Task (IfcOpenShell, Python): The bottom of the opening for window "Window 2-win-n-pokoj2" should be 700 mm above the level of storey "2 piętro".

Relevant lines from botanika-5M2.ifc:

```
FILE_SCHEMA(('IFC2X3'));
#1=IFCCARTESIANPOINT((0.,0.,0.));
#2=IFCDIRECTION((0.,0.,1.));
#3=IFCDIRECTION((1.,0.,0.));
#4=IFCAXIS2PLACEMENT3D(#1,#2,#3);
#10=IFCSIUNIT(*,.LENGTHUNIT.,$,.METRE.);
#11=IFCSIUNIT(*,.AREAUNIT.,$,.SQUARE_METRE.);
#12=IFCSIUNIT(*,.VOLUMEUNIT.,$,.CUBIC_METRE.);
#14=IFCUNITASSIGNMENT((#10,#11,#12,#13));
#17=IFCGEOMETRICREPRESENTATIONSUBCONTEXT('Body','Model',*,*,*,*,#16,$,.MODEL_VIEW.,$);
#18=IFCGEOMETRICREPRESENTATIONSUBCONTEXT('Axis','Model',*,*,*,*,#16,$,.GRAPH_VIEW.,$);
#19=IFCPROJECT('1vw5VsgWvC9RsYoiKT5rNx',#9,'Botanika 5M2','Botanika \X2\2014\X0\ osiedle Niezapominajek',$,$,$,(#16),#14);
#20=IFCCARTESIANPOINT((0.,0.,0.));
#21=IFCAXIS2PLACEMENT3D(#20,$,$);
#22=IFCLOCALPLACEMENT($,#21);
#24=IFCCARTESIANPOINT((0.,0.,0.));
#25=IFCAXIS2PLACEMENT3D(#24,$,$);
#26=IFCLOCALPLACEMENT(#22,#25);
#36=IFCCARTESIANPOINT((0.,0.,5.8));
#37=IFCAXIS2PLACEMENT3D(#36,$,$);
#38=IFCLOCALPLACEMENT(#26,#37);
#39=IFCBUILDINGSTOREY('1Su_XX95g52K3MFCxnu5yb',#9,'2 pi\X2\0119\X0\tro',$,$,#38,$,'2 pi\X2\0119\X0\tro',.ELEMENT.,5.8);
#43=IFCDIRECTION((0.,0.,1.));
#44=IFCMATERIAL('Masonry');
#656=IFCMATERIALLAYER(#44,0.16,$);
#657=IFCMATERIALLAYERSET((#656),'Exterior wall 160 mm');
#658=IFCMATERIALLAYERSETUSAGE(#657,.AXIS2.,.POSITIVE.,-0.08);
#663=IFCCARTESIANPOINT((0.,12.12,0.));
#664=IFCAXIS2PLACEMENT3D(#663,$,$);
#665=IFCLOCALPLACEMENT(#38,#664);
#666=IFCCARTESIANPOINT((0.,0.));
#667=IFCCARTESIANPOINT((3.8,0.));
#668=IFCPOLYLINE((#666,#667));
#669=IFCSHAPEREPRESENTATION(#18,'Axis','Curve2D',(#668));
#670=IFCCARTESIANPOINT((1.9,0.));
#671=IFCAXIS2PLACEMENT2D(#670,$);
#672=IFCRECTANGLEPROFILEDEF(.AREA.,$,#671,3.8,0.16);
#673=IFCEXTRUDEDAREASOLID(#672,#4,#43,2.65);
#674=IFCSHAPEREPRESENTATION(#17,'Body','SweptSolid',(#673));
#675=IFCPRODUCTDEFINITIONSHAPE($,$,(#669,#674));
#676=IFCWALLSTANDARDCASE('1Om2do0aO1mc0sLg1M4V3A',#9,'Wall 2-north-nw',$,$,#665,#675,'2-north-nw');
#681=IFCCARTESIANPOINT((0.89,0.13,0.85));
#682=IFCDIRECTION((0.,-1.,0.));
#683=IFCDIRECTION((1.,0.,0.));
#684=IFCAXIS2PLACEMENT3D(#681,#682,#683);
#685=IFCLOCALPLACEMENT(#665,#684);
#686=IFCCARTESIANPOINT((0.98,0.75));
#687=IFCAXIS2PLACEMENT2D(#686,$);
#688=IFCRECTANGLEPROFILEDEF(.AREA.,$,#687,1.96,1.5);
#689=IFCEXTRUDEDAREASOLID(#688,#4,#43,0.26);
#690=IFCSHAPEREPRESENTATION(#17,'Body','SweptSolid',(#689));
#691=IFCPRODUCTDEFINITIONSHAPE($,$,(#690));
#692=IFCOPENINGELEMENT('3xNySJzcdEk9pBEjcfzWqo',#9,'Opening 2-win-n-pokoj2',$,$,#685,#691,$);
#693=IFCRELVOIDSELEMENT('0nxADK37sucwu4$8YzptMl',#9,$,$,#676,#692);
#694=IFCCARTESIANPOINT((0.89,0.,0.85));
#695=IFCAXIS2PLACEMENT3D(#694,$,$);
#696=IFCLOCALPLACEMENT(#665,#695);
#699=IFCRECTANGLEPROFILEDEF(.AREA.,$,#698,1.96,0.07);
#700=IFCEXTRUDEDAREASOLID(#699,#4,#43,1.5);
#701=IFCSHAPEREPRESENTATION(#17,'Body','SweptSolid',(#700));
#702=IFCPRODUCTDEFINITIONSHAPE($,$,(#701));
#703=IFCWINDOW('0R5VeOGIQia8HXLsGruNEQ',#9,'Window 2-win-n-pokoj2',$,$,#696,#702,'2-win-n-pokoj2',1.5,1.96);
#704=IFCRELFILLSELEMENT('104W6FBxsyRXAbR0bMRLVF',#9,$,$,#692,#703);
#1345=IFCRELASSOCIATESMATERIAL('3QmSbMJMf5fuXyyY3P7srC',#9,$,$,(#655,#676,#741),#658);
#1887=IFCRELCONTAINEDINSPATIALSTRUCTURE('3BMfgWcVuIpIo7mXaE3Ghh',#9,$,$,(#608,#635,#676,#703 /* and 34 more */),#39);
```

```python
import numpy as np
import ifcopenshell
import ifcopenshell.api.geometry
import ifcopenshell.geom
import ifcopenshell.util.element
import ifcopenshell.util.placement
import ifcopenshell.util.shape
import ifcopenshell.util.unit

model = ifcopenshell.open("botanika-5M2.ifc")
unit_scale = ifcopenshell.util.unit.calculate_unit_scale(model)

window = model.by_guid("0R5VeOGIQia8HXLsGruNEQ")
opening = window.FillsVoids[0].RelatingOpeningElement
storey = ifcopenshell.util.element.get_container(window, ifc_class="IfcBuildingStorey")
level = ifcopenshell.util.placement.get_local_placement(storey.ObjectPlacement)[2, 3]

# The opening's origin need not be at the sill, so measure its lowest point.
shape = ifcopenshell.geom.create_shape(ifcopenshell.geom.settings(), opening)
bottom = ifcopenshell.util.shape.get_shape_bottom_elevation(shape, shape.geometry) / unit_scale
dz = level + 0.7 / unit_scale - bottom

shift = np.array([0.0, 0.0, dz])
# The window is not placed relative to its opening, so move both.
for product in (opening, window):
    matrix = ifcopenshell.util.placement.get_local_placement(product.ObjectPlacement)
    matrix[:3, 3] += shift
    ifcopenshell.api.geometry.edit_object_placement(model, product=product, matrix=matrix, is_si=False)

print(f"moved by {dz * unit_scale:+.3f} m")

model.write("botanika-5M2_rev.ifc")
```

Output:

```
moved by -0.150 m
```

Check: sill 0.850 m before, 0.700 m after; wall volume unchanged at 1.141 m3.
